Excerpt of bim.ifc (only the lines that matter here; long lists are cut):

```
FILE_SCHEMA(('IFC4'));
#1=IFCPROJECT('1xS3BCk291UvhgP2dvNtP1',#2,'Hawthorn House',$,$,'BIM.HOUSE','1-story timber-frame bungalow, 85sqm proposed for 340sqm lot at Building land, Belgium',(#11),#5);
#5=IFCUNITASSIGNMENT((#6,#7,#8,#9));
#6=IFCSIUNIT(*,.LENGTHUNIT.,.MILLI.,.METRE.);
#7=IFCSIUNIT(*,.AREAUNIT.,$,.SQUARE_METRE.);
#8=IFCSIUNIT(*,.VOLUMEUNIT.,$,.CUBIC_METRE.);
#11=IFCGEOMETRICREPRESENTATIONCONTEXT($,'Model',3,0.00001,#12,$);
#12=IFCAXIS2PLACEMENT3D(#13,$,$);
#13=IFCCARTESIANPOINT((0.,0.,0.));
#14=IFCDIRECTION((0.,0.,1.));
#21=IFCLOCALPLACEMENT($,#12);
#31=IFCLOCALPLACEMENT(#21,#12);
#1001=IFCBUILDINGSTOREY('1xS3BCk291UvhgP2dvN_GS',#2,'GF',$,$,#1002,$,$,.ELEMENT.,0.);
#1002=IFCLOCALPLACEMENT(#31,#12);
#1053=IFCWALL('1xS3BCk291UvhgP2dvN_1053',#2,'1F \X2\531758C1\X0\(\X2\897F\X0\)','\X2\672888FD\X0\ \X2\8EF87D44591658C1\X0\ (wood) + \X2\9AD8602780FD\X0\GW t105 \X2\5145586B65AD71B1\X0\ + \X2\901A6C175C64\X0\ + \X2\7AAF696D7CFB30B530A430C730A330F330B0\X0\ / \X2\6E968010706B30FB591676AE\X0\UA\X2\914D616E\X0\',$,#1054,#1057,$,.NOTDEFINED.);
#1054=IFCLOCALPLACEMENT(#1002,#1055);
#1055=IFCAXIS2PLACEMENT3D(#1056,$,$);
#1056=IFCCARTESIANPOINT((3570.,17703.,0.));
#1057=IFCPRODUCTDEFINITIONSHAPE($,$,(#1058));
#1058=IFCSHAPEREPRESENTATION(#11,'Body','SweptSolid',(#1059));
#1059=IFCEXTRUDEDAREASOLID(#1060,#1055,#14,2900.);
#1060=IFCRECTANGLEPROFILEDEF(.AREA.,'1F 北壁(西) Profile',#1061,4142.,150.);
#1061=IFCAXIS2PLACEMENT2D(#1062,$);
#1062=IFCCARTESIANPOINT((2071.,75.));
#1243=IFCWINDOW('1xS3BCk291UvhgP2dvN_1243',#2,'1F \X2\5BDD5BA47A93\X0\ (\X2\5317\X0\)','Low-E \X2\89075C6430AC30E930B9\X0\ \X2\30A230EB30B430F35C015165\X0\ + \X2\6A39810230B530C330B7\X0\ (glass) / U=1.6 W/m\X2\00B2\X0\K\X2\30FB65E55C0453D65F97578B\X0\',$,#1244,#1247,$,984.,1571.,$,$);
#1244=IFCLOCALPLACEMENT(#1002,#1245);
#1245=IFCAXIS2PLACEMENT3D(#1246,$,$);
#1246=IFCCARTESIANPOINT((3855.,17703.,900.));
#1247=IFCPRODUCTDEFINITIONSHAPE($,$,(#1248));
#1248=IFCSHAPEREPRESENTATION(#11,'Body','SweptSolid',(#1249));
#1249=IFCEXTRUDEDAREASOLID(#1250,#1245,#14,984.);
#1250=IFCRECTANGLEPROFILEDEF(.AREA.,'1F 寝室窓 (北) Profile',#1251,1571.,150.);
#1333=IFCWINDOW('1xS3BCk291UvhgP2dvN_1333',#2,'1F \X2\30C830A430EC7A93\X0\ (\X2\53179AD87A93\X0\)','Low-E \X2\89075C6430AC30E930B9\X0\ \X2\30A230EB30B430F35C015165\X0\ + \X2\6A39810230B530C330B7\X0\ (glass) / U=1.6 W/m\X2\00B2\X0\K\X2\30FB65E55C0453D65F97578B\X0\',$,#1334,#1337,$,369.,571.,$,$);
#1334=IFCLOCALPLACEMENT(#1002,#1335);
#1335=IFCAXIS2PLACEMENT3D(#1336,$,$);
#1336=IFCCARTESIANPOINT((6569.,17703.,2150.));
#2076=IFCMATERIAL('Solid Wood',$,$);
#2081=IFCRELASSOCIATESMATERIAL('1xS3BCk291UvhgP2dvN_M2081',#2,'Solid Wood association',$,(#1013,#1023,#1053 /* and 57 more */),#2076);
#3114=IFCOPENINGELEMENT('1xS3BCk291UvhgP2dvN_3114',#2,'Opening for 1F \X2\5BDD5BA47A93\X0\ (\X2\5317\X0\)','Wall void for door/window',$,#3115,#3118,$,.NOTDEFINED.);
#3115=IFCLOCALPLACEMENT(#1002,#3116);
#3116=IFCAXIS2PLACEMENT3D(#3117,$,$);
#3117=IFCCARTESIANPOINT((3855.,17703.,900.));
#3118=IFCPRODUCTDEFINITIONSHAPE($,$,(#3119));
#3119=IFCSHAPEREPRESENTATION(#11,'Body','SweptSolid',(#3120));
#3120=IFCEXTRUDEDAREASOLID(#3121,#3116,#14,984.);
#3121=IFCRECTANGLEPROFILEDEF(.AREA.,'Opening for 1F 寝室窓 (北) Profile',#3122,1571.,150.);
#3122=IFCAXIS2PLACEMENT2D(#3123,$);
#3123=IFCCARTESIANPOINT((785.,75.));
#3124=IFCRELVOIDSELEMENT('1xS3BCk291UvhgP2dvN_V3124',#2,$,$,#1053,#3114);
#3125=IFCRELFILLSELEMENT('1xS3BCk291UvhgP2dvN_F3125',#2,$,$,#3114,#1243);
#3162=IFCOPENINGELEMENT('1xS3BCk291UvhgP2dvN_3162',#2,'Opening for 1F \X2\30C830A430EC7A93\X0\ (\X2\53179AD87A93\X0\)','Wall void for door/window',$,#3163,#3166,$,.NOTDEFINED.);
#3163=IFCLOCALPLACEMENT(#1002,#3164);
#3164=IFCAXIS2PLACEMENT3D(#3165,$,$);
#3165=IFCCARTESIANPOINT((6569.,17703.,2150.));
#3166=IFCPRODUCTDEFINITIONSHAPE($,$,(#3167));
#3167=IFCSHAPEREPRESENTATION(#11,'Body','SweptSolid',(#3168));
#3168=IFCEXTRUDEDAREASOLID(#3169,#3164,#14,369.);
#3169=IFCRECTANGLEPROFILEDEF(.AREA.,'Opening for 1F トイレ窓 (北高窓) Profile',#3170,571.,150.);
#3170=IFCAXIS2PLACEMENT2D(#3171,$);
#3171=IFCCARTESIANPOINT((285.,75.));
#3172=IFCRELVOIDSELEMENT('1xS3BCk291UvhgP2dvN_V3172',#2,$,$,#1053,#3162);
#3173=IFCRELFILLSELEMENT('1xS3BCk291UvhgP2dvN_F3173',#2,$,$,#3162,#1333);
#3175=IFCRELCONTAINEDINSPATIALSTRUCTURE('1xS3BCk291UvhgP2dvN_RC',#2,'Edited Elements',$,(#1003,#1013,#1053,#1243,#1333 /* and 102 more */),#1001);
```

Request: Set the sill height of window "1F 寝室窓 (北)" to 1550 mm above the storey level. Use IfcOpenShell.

```python
import numpy as np
import ifcopenshell
import ifcopenshell.api.geometry
import ifcopenshell.geom
import ifcopenshell.util.element
import ifcopenshell.util.placement
import ifcopenshell.util.shape
import ifcopenshell.util.unit

model = ifcopenshell.open("bim.ifc")
unit_scale = ifcopenshell.util.unit.calculate_unit_scale(model)

window = model.by_guid("1xS3BCk291UvhgP2dvN_1243")
opening = window.FillsVoids[0].RelatingOpeningElement
storey = ifcopenshell.util.element.get_container(window, ifc_class="IfcBuildingStorey")
level = ifcopenshell.util.placement.get_local_placement(storey.ObjectPlacement)[2, 3]

# The opening's origin need not be at the sill, so measure its lowest point.
shape = ifcopenshell.geom.create_shape(ifcopenshell.geom.settings(), opening)
bottom = ifcopenshell.util.shape.get_shape_bottom_elevation(shape, shape.geometry) / unit_scale
dz = level + 1.55 / unit_scale - bottom

shift = np.array([0.0, 0.0, dz])
# The window is not placed relative to its opening, so move both.
for product in (opening, window):
    matrix = ifcopenshell.util.placement.get_local_placement(product.ObjectPlacement)
    matrix[:3, 3] += shift
    ifcopenshell.api.geometry.edit_object_placement(model, product=product, matrix=matrix, is_si=False)

print(f"moved by {dz * unit_scale:+.3f} m")

model.write("bim_updated.ifc")
```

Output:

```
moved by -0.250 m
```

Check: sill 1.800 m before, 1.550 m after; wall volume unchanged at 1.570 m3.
